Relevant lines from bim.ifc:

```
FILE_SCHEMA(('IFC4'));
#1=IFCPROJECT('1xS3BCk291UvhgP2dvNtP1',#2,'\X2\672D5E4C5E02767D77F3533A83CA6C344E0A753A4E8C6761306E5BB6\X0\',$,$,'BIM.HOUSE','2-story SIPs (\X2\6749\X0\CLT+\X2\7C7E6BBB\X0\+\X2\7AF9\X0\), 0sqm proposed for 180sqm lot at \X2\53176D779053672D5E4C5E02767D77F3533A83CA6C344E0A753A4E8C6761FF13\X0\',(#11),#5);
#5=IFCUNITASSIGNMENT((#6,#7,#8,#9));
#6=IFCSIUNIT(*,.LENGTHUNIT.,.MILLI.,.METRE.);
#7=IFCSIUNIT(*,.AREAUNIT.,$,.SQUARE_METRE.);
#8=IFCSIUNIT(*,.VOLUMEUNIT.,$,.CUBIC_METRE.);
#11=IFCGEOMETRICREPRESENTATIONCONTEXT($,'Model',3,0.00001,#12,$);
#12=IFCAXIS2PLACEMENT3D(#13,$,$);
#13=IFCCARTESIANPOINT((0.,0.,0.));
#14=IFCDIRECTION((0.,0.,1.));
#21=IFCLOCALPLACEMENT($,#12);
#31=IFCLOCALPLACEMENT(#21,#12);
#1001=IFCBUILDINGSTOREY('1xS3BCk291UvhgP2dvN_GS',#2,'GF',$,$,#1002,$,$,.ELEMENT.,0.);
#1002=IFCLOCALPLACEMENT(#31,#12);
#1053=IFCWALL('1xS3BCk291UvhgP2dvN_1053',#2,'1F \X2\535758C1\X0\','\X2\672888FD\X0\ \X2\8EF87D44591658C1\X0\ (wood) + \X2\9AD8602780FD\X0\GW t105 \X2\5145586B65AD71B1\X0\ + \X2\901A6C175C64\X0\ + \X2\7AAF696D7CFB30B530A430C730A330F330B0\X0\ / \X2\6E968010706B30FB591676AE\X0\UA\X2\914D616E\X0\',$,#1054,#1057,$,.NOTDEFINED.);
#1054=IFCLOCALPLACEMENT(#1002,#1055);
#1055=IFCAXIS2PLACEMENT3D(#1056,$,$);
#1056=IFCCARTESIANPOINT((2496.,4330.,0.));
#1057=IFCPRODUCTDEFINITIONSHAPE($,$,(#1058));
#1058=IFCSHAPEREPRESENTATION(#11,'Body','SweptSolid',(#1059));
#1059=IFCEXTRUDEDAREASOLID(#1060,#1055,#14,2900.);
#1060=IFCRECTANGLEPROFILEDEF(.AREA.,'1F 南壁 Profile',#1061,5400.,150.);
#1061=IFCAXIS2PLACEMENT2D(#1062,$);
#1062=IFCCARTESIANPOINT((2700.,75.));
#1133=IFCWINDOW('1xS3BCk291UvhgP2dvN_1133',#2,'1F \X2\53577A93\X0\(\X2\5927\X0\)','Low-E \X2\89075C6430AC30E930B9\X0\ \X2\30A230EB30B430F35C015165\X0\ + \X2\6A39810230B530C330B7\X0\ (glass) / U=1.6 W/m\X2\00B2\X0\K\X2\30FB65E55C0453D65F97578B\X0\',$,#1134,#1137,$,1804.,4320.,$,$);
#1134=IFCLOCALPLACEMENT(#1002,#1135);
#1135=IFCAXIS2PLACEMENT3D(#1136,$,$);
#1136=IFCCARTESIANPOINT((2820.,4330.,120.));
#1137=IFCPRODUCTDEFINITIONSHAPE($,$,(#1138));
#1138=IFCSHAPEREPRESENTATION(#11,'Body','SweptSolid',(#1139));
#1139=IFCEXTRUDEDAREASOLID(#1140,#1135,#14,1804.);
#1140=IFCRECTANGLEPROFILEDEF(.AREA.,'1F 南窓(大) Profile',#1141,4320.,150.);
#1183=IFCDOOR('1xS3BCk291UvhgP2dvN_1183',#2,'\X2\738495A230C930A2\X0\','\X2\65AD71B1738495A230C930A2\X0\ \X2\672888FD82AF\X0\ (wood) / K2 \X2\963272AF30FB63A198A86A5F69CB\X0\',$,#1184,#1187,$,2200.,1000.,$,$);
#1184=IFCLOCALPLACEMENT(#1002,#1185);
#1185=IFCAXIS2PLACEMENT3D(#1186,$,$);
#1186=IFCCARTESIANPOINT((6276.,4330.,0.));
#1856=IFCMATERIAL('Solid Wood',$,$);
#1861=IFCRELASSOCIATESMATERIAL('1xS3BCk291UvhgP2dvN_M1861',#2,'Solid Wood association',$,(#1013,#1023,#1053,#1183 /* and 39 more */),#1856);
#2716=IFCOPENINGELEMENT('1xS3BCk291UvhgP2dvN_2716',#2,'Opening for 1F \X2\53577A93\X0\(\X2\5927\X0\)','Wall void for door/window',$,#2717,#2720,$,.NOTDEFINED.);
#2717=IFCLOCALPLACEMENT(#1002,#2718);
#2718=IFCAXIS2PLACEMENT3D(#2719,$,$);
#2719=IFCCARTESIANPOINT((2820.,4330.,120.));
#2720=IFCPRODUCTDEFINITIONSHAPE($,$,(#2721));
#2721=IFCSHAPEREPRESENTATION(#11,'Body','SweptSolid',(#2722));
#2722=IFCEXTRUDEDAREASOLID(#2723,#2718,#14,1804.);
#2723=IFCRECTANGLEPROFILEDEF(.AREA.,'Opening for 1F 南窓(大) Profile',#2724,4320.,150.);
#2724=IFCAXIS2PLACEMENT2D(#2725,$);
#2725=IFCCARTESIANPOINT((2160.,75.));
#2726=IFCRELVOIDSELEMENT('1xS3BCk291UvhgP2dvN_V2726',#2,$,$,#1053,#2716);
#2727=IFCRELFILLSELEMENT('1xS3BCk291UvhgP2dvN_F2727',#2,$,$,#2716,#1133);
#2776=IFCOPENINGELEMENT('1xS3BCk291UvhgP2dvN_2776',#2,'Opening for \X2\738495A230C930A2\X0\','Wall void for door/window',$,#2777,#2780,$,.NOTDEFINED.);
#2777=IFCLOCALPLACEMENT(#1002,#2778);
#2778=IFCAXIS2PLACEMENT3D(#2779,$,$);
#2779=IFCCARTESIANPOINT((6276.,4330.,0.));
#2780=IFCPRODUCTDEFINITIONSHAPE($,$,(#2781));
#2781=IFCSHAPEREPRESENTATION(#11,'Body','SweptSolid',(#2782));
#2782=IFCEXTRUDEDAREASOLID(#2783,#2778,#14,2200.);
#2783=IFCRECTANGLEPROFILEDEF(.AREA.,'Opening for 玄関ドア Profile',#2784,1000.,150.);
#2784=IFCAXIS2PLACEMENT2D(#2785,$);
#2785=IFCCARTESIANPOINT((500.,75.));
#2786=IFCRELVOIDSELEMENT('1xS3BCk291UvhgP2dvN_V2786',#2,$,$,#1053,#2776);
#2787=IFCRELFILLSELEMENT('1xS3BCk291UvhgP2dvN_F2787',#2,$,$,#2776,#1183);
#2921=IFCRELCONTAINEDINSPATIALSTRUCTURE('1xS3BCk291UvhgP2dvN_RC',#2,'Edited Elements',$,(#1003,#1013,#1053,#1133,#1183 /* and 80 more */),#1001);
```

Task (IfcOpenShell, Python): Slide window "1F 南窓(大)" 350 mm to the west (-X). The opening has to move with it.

```python
import ifcopenshell
import ifcopenshell.api.geometry
import ifcopenshell.util.placement

model = ifcopenshell.open("bim.ifc")

window = model.by_guid("1xS3BCk291UvhgP2dvN_1133")
opening = window.FillsVoids[0].RelatingOpeningElement
wall = opening.VoidsElements[0].RelatingBuildingElement

wall_matrix = ifcopenshell.util.placement.get_local_placement(wall.ObjectPlacement)
shift = wall_matrix[:3, 0] * -350.0
before = ifcopenshell.util.placement.get_local_placement(window.ObjectPlacement)[:3, 3].copy()

# The window is not placed relative to its opening, so move both.
for product in (opening, window):
    matrix = ifcopenshell.util.placement.get_local_placement(product.ObjectPlacement)
    matrix[:3, 3] += shift
    ifcopenshell.api.geometry.edit_object_placement(model, product=product, matrix=matrix, is_si=False)

after = ifcopenshell.util.placement.get_local_placement(window.ObjectPlacement)[:3, 3]
print("window moved by", (after - before).round(3) + 0.0)

model.write("bim_updated.ifc")
```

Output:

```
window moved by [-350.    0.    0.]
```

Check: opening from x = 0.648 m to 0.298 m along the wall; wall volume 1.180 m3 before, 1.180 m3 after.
